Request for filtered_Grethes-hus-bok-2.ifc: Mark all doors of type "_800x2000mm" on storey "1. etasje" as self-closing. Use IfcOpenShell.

First a look at what the model holds.

```python
import ifcopenshell
import ifcopenshell.util.element

model = ifcopenshell.open("filtered_Grethes-hus-bok-2.ifc")
print(model.schema)
storey = next(s for s in model.by_type("IfcBuildingStorey") if s.Name == "1. etasje")
doors = [e for e in ifcopenshell.util.element.get_decomposition(storey) if e.is_a("IfcDoor")]
seen = {}
for e in doors:
    element_type = ifcopenshell.util.element.get_type(e)
    key = (element_type.Name if element_type != e and element_type else None, ifcopenshell.util.element.get_pset(e, "Pset_DoorCommon", "SelfClosing"))
    seen[key] = seen.get(key, 0) + 1
for (name, value), count in sorted(seen.items(), key=str):
    print(count, "x", name, "|", value)
```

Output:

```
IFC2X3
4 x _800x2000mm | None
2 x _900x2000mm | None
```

```python
import ifcopenshell
import ifcopenshell.api.pset
import ifcopenshell.util.element

model = ifcopenshell.open("filtered_Grethes-hus-bok-2.ifc")

storey = next(s for s in model.by_type("IfcBuildingStorey") if s.Name == "1. etasje")
doors = [e for e in ifcopenshell.util.element.get_decomposition(storey) if e.is_a("IfcDoor")]

count = 0
for e in doors:
    element_type = ifcopenshell.util.element.get_type(e)
    if element_type in (None, e) or element_type.Name != "_800x2000mm":
        continue
    # add_pset returns the element's existing set when there is one.
    pset = ifcopenshell.api.pset.add_pset(model, product=e, name="Pset_DoorCommon")
    ifcopenshell.api.pset.edit_pset(model, pset=pset, properties={"SelfClosing": True})
    count += 1

print(count, "doors updated")

model.write("filtered_Grethes-hus-bok-2-out.ifc")
```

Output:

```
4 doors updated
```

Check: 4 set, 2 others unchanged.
